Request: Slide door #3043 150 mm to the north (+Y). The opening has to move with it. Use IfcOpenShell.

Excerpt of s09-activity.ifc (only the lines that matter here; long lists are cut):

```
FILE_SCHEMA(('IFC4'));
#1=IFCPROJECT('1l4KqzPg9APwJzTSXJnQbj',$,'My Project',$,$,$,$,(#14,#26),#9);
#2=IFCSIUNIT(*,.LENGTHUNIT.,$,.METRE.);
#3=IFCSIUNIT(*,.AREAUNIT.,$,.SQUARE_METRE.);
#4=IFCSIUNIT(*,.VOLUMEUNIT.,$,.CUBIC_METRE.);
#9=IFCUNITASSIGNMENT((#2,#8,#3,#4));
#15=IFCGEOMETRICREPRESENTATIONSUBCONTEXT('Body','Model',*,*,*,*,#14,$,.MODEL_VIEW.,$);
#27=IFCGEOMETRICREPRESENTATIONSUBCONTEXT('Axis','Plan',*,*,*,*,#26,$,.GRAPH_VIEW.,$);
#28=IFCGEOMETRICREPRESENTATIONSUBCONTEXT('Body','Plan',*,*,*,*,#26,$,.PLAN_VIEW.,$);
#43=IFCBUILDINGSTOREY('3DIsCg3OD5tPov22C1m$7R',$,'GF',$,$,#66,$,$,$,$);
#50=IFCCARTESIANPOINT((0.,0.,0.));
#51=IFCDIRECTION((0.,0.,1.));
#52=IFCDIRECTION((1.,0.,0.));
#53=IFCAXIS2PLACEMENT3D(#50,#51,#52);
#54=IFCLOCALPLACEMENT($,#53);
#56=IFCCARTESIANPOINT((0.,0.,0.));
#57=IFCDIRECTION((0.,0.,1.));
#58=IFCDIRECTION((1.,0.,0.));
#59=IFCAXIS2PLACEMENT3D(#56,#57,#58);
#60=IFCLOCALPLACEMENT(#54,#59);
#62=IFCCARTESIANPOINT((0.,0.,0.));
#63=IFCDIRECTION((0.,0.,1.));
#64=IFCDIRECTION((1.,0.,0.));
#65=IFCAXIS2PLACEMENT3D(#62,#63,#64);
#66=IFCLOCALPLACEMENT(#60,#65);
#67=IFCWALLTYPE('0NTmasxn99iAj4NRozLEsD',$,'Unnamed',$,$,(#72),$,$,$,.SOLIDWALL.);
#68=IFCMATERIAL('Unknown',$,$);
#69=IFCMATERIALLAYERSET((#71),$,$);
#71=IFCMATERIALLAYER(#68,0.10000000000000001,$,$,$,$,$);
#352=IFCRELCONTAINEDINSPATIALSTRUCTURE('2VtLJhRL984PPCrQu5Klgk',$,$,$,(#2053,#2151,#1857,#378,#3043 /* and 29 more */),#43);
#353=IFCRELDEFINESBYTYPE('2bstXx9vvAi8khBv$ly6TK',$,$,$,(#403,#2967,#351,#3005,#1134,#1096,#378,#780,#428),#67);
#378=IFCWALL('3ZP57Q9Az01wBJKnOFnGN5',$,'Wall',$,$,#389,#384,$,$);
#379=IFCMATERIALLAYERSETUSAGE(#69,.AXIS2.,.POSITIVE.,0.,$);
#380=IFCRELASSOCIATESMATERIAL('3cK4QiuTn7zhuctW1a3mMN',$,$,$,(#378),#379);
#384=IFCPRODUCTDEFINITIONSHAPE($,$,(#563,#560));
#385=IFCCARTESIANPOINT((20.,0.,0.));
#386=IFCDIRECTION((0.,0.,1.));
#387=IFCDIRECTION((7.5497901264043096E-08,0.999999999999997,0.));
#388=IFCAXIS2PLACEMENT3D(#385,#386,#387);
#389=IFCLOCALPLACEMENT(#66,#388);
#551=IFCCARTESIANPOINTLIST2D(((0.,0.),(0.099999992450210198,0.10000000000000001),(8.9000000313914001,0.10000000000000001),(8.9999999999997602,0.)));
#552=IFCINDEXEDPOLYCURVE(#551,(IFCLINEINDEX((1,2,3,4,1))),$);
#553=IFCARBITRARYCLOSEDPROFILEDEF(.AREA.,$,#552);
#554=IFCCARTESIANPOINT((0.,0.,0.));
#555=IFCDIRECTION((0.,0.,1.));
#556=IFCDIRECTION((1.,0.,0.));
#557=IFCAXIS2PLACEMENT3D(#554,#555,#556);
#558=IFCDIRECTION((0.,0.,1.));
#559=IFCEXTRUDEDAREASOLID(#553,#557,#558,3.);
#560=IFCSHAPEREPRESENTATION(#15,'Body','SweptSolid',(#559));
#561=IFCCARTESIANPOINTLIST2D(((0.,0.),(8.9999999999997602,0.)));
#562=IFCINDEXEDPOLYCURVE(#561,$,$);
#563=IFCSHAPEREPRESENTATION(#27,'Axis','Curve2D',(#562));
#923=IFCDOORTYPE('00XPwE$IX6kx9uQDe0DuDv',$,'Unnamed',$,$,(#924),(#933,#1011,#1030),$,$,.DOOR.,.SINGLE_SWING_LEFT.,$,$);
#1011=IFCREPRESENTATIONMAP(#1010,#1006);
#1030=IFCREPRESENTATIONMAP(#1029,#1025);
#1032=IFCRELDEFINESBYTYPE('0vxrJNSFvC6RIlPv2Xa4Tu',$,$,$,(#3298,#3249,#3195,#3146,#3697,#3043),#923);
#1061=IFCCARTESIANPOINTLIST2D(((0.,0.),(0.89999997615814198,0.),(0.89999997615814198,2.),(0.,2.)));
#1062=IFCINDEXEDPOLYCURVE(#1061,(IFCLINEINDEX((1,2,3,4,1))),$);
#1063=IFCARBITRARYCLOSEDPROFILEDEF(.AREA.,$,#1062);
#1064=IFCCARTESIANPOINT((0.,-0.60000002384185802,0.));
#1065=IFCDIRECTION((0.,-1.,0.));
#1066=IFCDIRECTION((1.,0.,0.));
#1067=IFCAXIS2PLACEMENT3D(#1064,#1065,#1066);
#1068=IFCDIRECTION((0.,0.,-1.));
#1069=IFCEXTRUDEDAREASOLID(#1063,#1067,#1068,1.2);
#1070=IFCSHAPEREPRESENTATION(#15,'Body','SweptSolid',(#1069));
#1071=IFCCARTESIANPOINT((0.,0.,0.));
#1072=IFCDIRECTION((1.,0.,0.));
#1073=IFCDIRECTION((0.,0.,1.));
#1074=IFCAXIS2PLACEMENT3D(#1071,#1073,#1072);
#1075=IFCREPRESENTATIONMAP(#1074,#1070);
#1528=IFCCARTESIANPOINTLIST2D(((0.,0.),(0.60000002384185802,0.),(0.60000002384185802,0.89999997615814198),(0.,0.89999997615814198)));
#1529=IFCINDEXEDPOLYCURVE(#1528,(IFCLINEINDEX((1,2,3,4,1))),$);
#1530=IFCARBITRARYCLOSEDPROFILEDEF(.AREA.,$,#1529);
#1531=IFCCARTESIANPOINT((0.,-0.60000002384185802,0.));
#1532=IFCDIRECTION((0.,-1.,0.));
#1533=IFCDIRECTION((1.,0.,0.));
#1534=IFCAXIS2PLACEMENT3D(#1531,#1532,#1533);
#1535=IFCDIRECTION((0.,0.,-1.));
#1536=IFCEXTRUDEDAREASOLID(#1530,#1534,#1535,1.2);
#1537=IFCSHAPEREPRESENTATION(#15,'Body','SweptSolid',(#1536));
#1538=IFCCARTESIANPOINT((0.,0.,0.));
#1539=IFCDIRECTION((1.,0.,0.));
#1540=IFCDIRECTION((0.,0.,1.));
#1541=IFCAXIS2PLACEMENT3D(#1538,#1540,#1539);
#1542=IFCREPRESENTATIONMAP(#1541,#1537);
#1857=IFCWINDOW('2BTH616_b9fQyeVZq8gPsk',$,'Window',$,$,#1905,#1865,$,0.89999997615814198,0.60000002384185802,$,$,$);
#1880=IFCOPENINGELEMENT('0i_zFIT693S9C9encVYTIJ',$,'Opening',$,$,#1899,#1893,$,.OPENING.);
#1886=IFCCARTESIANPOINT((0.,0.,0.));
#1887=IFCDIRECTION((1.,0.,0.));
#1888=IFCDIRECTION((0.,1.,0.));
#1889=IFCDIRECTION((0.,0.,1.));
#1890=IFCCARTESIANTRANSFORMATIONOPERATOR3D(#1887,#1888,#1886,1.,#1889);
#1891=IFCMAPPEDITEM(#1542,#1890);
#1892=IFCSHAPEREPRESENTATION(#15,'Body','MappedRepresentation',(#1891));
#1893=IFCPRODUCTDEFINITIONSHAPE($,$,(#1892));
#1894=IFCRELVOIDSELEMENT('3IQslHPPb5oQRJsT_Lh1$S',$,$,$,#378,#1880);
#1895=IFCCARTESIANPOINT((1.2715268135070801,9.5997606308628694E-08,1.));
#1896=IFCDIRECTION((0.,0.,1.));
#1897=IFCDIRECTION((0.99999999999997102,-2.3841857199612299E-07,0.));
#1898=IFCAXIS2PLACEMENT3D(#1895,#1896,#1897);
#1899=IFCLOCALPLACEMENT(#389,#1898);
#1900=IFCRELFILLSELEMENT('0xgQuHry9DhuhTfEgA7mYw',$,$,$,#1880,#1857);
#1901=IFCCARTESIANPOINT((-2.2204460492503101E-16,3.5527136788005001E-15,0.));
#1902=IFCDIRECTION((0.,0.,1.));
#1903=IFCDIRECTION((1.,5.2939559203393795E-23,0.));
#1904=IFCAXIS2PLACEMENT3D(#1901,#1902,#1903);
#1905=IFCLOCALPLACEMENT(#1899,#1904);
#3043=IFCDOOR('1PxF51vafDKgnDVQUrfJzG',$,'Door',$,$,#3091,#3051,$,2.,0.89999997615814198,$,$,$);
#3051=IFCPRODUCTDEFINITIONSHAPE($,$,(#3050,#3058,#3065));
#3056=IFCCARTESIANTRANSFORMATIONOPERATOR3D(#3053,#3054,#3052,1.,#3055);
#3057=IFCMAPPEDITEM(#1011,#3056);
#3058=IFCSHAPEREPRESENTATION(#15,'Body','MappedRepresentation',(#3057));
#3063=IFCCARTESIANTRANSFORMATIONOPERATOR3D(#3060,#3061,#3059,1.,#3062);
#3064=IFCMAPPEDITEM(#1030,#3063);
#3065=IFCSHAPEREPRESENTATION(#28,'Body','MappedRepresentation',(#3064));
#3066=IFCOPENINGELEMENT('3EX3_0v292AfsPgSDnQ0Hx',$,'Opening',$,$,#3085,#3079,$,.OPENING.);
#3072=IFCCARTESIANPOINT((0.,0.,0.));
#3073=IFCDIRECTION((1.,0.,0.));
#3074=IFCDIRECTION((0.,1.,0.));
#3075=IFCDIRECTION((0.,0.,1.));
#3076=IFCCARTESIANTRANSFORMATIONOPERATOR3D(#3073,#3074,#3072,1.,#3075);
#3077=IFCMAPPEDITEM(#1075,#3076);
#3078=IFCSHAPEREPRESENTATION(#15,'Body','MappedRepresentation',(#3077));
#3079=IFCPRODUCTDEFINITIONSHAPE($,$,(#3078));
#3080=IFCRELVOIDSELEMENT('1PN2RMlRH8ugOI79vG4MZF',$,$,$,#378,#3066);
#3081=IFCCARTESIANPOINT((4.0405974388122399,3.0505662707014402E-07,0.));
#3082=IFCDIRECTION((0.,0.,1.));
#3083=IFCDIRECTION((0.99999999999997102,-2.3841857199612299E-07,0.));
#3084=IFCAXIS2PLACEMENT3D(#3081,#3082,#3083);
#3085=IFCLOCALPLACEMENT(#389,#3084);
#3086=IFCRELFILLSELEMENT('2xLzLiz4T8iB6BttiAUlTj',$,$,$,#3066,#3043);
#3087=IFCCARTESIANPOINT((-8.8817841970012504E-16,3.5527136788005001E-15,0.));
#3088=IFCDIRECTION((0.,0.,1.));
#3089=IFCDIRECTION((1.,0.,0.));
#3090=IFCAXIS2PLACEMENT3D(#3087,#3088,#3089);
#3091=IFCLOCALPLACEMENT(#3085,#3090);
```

```python
import ifcopenshell
import ifcopenshell.api.geometry
import ifcopenshell.util.placement

model = ifcopenshell.open("s09-activity.ifc")

door = model.by_guid("1PxF51vafDKgnDVQUrfJzG")
opening = door.FillsVoids[0].RelatingOpeningElement
wall = opening.VoidsElements[0].RelatingBuildingElement

wall_matrix = ifcopenshell.util.placement.get_local_placement(wall.ObjectPlacement)
shift = wall_matrix[:3, 0] * 0.15
before = ifcopenshell.util.placement.get_local_placement(door.ObjectPlacement)[:3, 3].copy()

# The door is placed relative to its opening, so it follows when the opening moves.
matrix = ifcopenshell.util.placement.get_local_placement(opening.ObjectPlacement)
matrix[:3, 3] += shift
ifcopenshell.api.geometry.edit_object_placement(
    model, product=opening, matrix=matrix, is_si=False, should_transform_children=True
)

after = ifcopenshell.util.placement.get_local_placement(door.ObjectPlacement)[:3, 3]
print("door moved by", (after - before).round(3) + 0.0)

model.write("s09-activity-out.ifc")
```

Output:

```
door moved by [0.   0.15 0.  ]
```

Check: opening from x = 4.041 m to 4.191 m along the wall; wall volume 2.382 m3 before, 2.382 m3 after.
